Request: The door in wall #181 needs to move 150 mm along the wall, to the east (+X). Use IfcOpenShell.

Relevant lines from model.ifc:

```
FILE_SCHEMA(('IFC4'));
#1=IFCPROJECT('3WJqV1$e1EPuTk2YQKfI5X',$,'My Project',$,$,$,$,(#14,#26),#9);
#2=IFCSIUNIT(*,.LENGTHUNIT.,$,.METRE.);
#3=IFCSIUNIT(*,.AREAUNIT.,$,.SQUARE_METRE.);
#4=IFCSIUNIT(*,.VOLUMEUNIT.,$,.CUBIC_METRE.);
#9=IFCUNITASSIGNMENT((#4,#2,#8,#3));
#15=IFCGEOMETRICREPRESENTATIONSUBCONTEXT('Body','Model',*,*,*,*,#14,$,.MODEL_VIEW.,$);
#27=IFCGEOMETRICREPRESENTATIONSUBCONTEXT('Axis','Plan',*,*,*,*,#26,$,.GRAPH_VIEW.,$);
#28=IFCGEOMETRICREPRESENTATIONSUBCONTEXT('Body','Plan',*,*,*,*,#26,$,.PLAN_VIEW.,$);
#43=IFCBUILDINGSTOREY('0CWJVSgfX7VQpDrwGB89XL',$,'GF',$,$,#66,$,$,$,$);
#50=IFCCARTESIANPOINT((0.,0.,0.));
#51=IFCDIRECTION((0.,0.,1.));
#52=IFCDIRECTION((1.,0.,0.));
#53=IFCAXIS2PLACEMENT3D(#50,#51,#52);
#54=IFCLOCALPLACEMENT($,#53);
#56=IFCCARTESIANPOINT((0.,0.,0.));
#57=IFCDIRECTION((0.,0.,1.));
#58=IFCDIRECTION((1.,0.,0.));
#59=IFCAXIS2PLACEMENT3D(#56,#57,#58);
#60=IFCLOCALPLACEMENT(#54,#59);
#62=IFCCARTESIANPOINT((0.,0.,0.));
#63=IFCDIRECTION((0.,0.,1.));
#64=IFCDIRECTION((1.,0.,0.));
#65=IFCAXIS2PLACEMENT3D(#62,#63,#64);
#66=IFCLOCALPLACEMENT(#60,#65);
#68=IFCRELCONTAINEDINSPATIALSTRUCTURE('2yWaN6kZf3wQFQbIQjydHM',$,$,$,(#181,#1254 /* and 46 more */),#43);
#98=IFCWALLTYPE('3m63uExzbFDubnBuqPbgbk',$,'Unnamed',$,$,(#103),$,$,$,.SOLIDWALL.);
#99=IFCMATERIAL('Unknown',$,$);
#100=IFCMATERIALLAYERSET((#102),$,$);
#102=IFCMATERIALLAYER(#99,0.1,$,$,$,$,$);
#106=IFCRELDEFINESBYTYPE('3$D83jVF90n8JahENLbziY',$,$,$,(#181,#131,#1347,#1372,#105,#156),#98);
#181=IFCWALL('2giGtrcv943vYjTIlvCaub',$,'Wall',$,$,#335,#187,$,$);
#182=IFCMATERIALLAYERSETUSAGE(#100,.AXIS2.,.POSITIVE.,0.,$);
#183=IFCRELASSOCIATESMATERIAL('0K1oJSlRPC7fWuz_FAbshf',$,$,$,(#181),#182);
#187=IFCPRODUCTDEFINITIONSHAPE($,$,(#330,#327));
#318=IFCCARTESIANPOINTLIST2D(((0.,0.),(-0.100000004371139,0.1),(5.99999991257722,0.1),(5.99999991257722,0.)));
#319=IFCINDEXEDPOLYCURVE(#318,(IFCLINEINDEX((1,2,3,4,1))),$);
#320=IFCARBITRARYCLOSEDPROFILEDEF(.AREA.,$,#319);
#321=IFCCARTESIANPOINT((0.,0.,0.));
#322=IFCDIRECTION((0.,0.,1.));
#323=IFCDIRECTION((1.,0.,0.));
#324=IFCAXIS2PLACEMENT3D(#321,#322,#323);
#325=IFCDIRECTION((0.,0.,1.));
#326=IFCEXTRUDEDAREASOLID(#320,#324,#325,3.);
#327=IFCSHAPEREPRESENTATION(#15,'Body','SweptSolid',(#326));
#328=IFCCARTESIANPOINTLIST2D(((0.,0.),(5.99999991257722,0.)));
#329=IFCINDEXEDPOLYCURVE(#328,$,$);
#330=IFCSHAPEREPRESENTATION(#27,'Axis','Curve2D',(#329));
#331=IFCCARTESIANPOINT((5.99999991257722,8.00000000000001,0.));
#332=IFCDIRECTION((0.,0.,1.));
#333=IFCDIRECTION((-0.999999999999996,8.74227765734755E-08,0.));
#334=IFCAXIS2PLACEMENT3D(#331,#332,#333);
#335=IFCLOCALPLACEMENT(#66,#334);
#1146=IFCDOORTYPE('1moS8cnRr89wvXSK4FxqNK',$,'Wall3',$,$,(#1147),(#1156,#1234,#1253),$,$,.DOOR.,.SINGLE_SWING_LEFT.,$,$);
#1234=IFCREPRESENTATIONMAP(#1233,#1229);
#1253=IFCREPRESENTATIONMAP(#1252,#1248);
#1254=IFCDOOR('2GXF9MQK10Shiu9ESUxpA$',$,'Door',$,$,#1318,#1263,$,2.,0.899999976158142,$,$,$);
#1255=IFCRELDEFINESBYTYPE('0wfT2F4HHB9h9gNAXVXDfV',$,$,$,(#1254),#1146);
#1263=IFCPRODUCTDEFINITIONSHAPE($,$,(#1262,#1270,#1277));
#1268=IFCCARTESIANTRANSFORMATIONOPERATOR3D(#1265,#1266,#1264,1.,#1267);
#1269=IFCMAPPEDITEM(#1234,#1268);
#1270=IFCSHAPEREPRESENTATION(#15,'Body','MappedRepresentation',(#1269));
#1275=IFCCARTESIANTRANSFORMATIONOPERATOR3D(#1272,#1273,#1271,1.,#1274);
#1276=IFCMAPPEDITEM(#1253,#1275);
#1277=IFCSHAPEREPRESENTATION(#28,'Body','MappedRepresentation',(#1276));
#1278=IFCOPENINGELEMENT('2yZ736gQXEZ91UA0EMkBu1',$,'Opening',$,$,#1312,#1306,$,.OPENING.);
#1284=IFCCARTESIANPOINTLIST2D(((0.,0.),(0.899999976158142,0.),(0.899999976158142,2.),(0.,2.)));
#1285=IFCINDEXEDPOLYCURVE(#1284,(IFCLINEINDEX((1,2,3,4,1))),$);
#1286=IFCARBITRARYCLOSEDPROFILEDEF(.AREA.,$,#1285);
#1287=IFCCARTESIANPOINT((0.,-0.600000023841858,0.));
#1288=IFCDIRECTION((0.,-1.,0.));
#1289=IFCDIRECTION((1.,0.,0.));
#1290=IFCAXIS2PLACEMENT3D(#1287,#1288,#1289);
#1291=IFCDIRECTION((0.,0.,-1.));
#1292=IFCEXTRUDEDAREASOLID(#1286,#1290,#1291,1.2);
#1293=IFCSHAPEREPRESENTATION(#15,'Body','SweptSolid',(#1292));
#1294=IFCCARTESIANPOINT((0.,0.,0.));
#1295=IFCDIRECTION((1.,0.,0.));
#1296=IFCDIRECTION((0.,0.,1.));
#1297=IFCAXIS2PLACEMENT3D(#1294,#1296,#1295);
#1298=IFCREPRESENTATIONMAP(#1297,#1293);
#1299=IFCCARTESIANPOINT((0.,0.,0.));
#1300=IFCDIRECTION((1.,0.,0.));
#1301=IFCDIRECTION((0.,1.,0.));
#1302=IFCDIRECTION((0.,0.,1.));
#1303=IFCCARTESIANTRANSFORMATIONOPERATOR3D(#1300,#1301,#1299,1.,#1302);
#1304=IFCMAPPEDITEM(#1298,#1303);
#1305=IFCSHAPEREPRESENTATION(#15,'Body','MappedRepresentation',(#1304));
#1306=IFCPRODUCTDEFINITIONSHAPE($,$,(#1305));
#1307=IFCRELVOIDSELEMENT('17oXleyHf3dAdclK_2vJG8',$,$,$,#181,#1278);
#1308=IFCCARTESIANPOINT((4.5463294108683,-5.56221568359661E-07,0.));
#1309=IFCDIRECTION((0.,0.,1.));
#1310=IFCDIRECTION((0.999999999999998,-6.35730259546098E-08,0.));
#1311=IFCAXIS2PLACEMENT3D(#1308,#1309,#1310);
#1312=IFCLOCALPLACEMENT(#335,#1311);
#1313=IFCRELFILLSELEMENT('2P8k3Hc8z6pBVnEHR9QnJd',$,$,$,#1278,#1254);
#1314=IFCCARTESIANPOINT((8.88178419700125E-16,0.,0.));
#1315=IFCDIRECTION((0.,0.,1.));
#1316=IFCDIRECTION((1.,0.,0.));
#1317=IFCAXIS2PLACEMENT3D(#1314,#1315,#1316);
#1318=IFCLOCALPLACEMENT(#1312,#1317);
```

```python
import ifcopenshell
import ifcopenshell.api.geometry
import ifcopenshell.util.placement

model = ifcopenshell.open("model.ifc")

door = model.by_guid("2GXF9MQK10Shiu9ESUxpA$")
opening = door.FillsVoids[0].RelatingOpeningElement
wall = opening.VoidsElements[0].RelatingBuildingElement

wall_matrix = ifcopenshell.util.placement.get_local_placement(wall.ObjectPlacement)
shift = wall_matrix[:3, 0] * -0.15
before = ifcopenshell.util.placement.get_local_placement(door.ObjectPlacement)[:3, 3].copy()

# The door is placed relative to its opening, so it follows when the opening moves.
matrix = ifcopenshell.util.placement.get_local_placement(opening.ObjectPlacement)
matrix[:3, 3] += shift
ifcopenshell.api.geometry.edit_object_placement(
    model, product=opening, matrix=matrix, is_si=False, should_transform_children=True
)

after = ifcopenshell.util.placement.get_local_placement(door.ObjectPlacement)[:3, 3]
print("door moved by", (after - before).round(3) + 0.0)

model.write("model_v2.ifc")
```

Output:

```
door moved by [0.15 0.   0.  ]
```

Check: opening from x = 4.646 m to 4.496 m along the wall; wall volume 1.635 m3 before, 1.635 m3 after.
